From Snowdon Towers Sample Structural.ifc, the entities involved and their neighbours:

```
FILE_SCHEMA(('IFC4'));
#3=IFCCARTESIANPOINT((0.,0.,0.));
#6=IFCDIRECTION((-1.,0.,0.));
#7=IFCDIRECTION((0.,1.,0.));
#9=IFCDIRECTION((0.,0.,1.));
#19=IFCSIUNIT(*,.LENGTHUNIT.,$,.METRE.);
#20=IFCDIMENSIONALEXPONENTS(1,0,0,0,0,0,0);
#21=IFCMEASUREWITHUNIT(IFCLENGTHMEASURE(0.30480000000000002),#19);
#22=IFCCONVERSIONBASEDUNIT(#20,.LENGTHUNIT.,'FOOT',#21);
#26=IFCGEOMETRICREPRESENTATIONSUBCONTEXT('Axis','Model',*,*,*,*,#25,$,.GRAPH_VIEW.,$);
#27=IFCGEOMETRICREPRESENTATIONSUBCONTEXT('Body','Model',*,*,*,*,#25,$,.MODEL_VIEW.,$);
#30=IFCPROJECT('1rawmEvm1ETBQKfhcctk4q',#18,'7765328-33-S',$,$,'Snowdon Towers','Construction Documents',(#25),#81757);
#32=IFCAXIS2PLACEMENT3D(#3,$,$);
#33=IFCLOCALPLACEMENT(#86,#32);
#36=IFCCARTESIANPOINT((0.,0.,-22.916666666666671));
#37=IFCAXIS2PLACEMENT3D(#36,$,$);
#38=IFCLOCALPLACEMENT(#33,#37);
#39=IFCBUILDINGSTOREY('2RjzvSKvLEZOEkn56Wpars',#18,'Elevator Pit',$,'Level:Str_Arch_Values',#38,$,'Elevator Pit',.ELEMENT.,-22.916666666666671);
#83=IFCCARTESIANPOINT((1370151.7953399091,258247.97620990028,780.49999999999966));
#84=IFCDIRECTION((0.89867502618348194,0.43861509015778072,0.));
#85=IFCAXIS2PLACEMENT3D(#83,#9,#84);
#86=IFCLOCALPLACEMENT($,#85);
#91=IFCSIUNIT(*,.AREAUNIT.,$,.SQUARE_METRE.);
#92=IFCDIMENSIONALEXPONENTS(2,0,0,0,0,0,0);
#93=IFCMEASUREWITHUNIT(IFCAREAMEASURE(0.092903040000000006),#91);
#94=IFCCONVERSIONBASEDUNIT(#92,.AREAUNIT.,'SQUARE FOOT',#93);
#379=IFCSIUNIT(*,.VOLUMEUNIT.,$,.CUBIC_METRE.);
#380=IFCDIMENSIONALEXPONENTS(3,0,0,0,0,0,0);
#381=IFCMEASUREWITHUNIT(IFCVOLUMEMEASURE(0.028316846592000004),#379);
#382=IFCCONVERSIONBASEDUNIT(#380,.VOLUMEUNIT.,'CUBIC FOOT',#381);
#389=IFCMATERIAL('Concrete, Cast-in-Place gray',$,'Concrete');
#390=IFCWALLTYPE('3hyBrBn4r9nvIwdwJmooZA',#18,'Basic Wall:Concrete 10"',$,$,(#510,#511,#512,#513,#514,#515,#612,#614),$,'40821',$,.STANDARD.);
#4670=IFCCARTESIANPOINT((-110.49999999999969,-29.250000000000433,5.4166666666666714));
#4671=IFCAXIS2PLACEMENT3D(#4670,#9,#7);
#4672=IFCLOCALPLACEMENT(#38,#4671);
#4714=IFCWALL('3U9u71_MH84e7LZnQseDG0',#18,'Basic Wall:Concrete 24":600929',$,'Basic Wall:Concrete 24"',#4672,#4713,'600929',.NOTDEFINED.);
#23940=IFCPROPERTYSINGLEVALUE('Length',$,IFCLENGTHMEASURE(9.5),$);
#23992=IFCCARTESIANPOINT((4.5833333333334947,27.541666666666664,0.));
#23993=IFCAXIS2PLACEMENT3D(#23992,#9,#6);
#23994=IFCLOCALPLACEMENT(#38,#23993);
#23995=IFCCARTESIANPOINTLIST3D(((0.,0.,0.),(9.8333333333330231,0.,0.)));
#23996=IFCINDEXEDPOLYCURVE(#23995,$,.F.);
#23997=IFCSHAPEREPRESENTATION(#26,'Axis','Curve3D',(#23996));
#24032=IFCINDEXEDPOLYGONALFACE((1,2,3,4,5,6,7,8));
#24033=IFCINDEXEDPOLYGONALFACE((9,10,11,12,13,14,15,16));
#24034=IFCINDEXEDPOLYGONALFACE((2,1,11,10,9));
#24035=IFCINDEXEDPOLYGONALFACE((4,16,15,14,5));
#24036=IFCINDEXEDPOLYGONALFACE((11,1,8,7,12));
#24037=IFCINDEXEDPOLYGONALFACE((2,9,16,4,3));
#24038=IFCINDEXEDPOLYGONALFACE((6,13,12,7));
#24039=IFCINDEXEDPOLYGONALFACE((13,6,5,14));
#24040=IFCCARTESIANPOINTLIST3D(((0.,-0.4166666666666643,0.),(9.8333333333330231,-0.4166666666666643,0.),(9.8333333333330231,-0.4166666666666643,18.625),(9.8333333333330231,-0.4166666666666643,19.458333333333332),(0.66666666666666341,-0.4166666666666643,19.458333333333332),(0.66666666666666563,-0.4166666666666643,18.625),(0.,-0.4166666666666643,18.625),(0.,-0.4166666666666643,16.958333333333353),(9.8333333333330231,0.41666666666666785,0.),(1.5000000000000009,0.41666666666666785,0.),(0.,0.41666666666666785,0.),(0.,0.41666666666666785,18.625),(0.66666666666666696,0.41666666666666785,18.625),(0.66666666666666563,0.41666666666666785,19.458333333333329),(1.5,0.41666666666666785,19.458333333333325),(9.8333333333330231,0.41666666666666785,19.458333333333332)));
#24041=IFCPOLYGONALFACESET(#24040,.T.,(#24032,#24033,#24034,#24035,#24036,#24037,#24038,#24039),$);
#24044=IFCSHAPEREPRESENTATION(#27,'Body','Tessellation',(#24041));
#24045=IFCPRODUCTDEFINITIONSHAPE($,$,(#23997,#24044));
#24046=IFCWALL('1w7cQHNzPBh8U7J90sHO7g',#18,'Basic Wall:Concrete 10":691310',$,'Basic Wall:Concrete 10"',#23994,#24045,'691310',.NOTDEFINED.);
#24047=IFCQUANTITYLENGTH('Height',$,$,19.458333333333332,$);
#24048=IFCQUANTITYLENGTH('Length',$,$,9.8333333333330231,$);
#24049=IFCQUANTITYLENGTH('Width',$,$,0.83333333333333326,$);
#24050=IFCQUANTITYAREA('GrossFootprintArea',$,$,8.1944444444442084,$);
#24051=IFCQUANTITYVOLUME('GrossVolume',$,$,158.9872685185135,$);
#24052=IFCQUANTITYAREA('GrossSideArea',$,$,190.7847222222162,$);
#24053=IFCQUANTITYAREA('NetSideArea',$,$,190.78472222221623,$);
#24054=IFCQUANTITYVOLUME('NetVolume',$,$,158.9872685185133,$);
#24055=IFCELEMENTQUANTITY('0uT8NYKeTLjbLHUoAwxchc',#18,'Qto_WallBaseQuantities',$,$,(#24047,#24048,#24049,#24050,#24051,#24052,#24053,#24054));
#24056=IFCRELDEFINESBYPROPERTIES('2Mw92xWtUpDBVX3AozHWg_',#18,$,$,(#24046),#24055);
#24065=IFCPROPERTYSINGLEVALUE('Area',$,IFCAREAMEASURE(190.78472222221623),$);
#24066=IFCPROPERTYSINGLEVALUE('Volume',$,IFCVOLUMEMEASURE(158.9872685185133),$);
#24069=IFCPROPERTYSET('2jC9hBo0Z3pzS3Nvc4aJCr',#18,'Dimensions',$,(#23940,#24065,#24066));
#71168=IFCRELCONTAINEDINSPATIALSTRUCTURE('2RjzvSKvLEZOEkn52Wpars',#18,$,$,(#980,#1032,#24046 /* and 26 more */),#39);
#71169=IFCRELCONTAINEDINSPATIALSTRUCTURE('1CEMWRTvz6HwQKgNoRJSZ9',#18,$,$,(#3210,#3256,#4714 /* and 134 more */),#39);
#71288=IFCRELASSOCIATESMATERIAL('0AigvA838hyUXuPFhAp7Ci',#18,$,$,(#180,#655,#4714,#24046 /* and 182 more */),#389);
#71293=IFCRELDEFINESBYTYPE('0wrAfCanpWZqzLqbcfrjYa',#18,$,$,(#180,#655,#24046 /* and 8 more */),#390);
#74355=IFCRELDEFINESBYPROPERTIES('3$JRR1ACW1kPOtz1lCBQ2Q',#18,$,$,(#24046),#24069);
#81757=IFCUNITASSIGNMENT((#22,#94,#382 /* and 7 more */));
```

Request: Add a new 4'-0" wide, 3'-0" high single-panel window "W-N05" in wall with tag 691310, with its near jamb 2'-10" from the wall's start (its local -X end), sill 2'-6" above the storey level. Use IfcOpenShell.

```python
import numpy as np
import ifcopenshell
import ifcopenshell.api.feature
import ifcopenshell.api.geometry
import ifcopenshell.api.pset
import ifcopenshell.api.root
import ifcopenshell.api.spatial
import ifcopenshell.geom
import ifcopenshell.util.element
import ifcopenshell.util.placement
import ifcopenshell.util.representation
import ifcopenshell.util.shape
import ifcopenshell.util.unit

model = ifcopenshell.open("Snowdon Towers Sample Structural.ifc")
unit_scale = ifcopenshell.util.unit.calculate_unit_scale(model)
area_scale = ifcopenshell.util.unit.calculate_unit_scale(model, "AREAUNIT")
volume_scale = ifcopenshell.util.unit.calculate_unit_scale(model, "VOLUMEUNIT")
settings = ifcopenshell.geom.settings()


def volume(element):
    """Net volume in cubic metres, openings subtracted."""
    shape = ifcopenshell.geom.create_shape(settings, element)
    return ifcopenshell.util.shape.get_volume(shape.geometry)


wall = model.by_guid("1w7cQHNzPBh8U7J90sHO7g")
storey = ifcopenshell.util.element.get_container(wall, ifc_class="IfcBuildingStorey")
context = ifcopenshell.util.representation.get_context(model, "Model", "Body", "MODEL_VIEW")
before = volume(wall)

width, height, from_end, sill = 1.2192, 0.9144, 0.8636, 0.762  # metres

# The wall runs along its own X axis, and the end named is its -X end.
wall_shape = ifcopenshell.geom.create_shape(settings, wall)
x, y, z = ifcopenshell.util.shape.get_vertices(wall_shape.geometry).T
start = x.min() + from_end
face, thickness = float(y.min()), float(y.max() - y.min())
wall_matrix = ifcopenshell.util.placement.get_local_placement(wall.ObjectPlacement)
level = ifcopenshell.util.placement.get_local_placement(storey.ObjectPlacement)[2, 3]


def in_wall(x, y):
    """Placement at x, y metres in the wall's axes, at sill height."""
    matrix = wall_matrix.copy()
    matrix[:, 3] = wall_matrix @ np.array([x / unit_scale, y / unit_scale, 0.0, 1.0])
    matrix[2, 3] = level + sill / unit_scale
    return matrix


# Opening: a box that overshoots both wall faces by 50 mm.
opening = ifcopenshell.api.root.create_entity(model, ifc_class="IfcOpeningElement", predefined_type="OPENING")
box = ifcopenshell.api.geometry.add_wall_representation(
    model, context=context, length=width, height=height, thickness=thickness + 0.1
)
ifcopenshell.api.geometry.assign_representation(model, product=opening, representation=box)
ifcopenshell.api.geometry.edit_object_placement(model, product=opening, matrix=in_wall(start, face - 0.05), is_si=False)
ifcopenshell.api.feature.add_feature(model, feature=opening, element=wall)

window = ifcopenshell.api.root.create_entity(model, ifc_class="IfcWindow", name="W-N05", predefined_type="WINDOW")
window.OverallWidth, window.OverallHeight = width / unit_scale, height / unit_scale
window.PartitioningType = "SINGLE_PANEL"
body = ifcopenshell.api.geometry.add_window_representation(
    model,
    context=context,
    overall_width=window.OverallWidth,
    overall_height=window.OverallHeight,
    partition_type="SINGLE_PANEL",
)
ifcopenshell.api.geometry.assign_representation(model, product=window, representation=body)
ifcopenshell.api.spatial.assign_container(model, products=[window], relating_structure=storey)
ifcopenshell.api.feature.add_filling(model, opening=opening, element=window)

# Centre the window in the wall's thickness.
ifcopenshell.api.geometry.edit_object_placement(model, product=window, matrix=in_wall(start, face), is_si=False)
window_shape = ifcopenshell.geom.create_shape(settings, window)
depth = ifcopenshell.util.shape.get_vertices(window_shape.geometry)[:, 1]
offset = face + thickness / 2 - (depth.min() + depth.max()) / 2
ifcopenshell.api.geometry.edit_object_placement(model, product=window, matrix=in_wall(start, offset), is_si=False)

after = volume(wall)

# Update the wall's stored quantities.
qto = model.by_id(ifcopenshell.util.element.get_pset(wall, "Qto_WallBaseQuantities", should_inherit=False)["id"])
ifcopenshell.api.pset.edit_qto(model, qto=qto, properties={
    "NetSideArea": after / thickness / area_scale,
    "NetVolume": after / volume_scale,
})
pset = model.by_id(ifcopenshell.util.element.get_pset(wall, "Dimensions", should_inherit=False)["id"])
ifcopenshell.api.pset.edit_pset(model, pset=pset, properties={
    "Area": model.create_entity("IfcAreaMeasure", after / thickness / area_scale),
    "Volume": model.create_entity("IfcVolumeMeasure", after / volume_scale),
})

print(f"wall volume {before:.3f} -> {after:.3f} m3")

model.write("Snowdon Towers Sample Structural_v2.ifc")
```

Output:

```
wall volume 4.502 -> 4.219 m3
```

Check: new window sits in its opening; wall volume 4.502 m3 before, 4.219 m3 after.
